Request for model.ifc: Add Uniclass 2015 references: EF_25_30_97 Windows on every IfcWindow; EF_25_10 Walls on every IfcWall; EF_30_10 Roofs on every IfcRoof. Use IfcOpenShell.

First a look at what the model holds.

```python
import ifcopenshell

model = ifcopenshell.open("model.ifc")
print(model.schema)
print("classifications:", [c.Name for c in model.by_type("IfcClassification")])
for ifc_class in ("IfcDoor", "IfcRoof", "IfcStair", "IfcWall", "IfcWindow"):
    print(ifc_class, len(model.by_type(ifc_class)))
```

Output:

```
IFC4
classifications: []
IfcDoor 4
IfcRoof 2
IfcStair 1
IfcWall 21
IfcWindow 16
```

```python
import ifcopenshell
import ifcopenshell.api.classification

model = ifcopenshell.open("model.ifc")

system = ifcopenshell.api.classification.add_classification(model, classification="Uniclass 2015")

codes = {
    "IfcWindow": ("EF_25_30_97", "Windows"),
    "IfcWall": ("EF_25_10", "Walls"),
    "IfcRoof": ("EF_30_10", "Roofs"),
}
for ifc_class, (code, name) in codes.items():
    products = model.by_type(ifc_class)
    ifcopenshell.api.classification.add_reference(
        model, products=products, classification=system, identification=code, name=name
    )
    print(code, len(products))

model.write("model_rev.ifc")
```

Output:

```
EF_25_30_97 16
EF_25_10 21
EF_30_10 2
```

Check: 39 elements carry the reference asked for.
